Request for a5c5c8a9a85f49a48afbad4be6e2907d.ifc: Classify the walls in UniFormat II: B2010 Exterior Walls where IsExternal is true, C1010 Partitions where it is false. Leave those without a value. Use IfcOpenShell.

First a look at what the model holds.

```python
import ifcopenshell
import ifcopenshell.util.element

model = ifcopenshell.open("a5c5c8a9a85f49a48afbad4be6e2907d.ifc")
print(model.schema)
print("classifications:", [c.Name for c in model.by_type("IfcClassification")])
values = [ifcopenshell.util.element.get_pset(e, "Pset_WallCommon", "IsExternal") for e in model.by_type("IfcWall")]
for value in (True, False, None):
    print("IsExternal", value, values.count(value))
```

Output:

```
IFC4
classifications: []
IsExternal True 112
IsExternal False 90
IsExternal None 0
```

```python
import ifcopenshell
import ifcopenshell.api.classification
import ifcopenshell.util.element

model = ifcopenshell.open("a5c5c8a9a85f49a48afbad4be6e2907d.ifc")

system = ifcopenshell.api.classification.add_classification(model, classification="UniFormat II")

walls = model.by_type("IfcWall")
external = {e: ifcopenshell.util.element.get_pset(e, "Pset_WallCommon", "IsExternal") for e in walls}
for flag, code, name in ((True, "B2010", "Exterior Walls"), (False, "C1010", "Partitions")):
    products = [e for e in walls if external[e] is flag]
    ifcopenshell.api.classification.add_reference(
        model, products=products, classification=system, identification=code, name=name
    )
    print(code, len(products))

model.write("a5c5c8a9a85f49a48afbad4be6e2907d_updated.ifc")
```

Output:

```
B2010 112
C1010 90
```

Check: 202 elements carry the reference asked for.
